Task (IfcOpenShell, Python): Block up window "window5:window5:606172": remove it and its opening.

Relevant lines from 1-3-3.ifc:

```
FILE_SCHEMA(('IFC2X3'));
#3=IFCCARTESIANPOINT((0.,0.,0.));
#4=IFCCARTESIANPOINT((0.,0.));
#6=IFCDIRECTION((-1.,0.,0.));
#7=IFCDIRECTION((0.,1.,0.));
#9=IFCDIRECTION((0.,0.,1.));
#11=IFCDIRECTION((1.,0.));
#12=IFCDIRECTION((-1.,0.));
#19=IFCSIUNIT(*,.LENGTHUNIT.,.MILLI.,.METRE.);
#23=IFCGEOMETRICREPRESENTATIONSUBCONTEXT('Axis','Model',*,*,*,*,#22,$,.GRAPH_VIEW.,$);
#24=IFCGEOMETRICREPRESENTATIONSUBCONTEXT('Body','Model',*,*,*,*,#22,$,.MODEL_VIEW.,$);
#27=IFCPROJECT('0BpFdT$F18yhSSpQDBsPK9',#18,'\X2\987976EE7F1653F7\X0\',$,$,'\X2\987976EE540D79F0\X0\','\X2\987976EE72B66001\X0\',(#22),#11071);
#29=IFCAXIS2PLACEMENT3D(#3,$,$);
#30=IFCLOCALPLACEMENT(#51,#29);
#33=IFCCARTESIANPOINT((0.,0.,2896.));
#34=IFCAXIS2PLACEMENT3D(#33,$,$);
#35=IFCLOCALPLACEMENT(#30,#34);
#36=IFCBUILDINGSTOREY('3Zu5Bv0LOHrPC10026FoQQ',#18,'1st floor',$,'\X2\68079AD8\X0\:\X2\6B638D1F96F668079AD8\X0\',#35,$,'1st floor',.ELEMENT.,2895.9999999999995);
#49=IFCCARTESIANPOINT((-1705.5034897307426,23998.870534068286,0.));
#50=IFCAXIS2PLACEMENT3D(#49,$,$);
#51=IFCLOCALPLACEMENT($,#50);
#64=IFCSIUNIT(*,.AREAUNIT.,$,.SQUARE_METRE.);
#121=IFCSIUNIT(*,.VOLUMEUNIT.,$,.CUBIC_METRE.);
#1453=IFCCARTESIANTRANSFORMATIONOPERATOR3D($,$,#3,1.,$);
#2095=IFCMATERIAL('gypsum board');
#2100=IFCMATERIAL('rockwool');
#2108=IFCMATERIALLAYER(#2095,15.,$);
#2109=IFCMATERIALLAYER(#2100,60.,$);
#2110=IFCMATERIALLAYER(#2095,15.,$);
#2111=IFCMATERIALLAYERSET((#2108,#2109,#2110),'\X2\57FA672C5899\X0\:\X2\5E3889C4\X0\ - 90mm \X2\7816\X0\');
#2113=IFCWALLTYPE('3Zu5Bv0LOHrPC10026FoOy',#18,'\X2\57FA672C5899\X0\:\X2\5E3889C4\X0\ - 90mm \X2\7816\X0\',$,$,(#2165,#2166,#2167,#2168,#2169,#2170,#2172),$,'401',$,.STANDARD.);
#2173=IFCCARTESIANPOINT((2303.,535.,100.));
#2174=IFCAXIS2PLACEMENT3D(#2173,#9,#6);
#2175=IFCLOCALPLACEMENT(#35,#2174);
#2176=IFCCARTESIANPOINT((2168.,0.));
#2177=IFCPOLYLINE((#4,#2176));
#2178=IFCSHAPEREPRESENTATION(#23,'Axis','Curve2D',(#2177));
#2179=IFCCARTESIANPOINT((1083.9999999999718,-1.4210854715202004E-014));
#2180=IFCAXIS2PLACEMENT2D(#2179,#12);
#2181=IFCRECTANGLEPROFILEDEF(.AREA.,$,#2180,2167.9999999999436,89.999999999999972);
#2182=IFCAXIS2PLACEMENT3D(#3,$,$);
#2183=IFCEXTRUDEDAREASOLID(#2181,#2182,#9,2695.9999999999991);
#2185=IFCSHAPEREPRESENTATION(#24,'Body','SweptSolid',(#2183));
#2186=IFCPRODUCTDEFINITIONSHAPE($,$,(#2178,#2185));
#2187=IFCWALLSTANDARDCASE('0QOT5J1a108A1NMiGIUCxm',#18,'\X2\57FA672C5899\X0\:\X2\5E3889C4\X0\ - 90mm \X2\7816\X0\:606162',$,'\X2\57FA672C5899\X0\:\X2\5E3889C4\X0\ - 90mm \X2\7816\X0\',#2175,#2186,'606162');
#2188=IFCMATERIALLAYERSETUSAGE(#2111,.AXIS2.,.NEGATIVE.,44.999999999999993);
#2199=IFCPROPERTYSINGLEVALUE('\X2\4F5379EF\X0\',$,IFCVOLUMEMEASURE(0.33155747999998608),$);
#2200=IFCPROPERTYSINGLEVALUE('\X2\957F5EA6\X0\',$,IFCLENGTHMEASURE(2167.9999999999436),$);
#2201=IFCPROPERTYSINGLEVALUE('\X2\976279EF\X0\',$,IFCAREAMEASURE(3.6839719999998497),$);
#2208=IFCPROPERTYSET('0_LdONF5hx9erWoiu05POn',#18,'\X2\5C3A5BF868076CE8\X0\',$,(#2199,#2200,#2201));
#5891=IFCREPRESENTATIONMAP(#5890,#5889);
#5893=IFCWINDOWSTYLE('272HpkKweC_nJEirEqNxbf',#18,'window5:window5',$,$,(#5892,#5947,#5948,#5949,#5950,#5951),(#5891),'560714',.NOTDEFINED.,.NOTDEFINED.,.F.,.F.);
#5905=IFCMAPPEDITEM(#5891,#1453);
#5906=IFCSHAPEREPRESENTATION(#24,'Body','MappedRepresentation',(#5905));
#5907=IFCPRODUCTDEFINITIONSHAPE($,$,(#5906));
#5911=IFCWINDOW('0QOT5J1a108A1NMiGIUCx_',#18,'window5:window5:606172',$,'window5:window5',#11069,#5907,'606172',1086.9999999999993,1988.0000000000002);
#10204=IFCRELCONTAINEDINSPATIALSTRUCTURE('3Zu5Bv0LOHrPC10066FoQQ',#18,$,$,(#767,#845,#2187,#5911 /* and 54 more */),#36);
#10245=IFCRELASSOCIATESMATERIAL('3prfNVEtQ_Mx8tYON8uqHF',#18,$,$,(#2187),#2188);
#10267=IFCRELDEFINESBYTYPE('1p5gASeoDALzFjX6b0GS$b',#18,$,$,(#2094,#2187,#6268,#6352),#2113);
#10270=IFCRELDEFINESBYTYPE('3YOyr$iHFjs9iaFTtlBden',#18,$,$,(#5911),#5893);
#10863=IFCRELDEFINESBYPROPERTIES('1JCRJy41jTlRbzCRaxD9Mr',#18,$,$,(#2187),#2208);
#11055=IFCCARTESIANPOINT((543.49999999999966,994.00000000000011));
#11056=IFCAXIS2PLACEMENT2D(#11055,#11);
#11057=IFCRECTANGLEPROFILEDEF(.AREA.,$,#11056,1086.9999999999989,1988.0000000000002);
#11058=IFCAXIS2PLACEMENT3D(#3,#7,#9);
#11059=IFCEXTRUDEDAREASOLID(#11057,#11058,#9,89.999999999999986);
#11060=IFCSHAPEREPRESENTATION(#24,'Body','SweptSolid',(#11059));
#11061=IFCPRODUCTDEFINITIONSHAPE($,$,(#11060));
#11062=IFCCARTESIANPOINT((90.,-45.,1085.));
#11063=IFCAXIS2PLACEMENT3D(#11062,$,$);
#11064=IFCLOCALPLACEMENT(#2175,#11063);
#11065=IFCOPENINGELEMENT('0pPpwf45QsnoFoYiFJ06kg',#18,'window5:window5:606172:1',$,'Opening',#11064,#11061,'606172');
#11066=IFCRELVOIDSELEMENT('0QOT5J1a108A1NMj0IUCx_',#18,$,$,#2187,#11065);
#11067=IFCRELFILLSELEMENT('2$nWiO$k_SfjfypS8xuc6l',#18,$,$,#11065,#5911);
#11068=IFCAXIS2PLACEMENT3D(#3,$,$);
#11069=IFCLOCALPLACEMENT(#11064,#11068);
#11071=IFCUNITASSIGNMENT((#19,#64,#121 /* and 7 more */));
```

```python
import ifcopenshell
import ifcopenshell.api.feature
import ifcopenshell.api.pset
import ifcopenshell.api.root
import ifcopenshell.geom
import ifcopenshell.util.element
import ifcopenshell.util.shape
import ifcopenshell.util.unit

model = ifcopenshell.open("1-3-3.ifc")
area_scale = ifcopenshell.util.unit.calculate_unit_scale(model, "AREAUNIT")
volume_scale = ifcopenshell.util.unit.calculate_unit_scale(model, "VOLUMEUNIT")
settings = ifcopenshell.geom.settings()


def volume(element):
    """Net volume in cubic metres, openings subtracted."""
    shape = ifcopenshell.geom.create_shape(settings, element)
    return ifcopenshell.util.shape.get_volume(shape.geometry)


window = model.by_id(5911)
opening = window.FillsVoids[0].RelatingOpeningElement
wall = opening.VoidsElements[0].RelatingBuildingElement
before = volume(wall)

ifcopenshell.api.root.remove_product(model, product=window)
ifcopenshell.api.feature.remove_feature(model, feature=opening)

after = volume(wall)
thickness = 0.09  # wall thickness in metres

# Update the wall's stored quantities.
pset = model.by_id(ifcopenshell.util.element.get_pset(wall, "尺寸标注", should_inherit=False)["id"])
ifcopenshell.api.pset.edit_pset(model, pset=pset, properties={
    "体积": model.create_entity("IfcVolumeMeasure", after / volume_scale),
    "面积": model.create_entity("IfcAreaMeasure", after / thickness / area_scale),
})

print(f"wall volume {before:.3f} -> {after:.3f} m3")

model.write("1-3-3_updated.ifc")
```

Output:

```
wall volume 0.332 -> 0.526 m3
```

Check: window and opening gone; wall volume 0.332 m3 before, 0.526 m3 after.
